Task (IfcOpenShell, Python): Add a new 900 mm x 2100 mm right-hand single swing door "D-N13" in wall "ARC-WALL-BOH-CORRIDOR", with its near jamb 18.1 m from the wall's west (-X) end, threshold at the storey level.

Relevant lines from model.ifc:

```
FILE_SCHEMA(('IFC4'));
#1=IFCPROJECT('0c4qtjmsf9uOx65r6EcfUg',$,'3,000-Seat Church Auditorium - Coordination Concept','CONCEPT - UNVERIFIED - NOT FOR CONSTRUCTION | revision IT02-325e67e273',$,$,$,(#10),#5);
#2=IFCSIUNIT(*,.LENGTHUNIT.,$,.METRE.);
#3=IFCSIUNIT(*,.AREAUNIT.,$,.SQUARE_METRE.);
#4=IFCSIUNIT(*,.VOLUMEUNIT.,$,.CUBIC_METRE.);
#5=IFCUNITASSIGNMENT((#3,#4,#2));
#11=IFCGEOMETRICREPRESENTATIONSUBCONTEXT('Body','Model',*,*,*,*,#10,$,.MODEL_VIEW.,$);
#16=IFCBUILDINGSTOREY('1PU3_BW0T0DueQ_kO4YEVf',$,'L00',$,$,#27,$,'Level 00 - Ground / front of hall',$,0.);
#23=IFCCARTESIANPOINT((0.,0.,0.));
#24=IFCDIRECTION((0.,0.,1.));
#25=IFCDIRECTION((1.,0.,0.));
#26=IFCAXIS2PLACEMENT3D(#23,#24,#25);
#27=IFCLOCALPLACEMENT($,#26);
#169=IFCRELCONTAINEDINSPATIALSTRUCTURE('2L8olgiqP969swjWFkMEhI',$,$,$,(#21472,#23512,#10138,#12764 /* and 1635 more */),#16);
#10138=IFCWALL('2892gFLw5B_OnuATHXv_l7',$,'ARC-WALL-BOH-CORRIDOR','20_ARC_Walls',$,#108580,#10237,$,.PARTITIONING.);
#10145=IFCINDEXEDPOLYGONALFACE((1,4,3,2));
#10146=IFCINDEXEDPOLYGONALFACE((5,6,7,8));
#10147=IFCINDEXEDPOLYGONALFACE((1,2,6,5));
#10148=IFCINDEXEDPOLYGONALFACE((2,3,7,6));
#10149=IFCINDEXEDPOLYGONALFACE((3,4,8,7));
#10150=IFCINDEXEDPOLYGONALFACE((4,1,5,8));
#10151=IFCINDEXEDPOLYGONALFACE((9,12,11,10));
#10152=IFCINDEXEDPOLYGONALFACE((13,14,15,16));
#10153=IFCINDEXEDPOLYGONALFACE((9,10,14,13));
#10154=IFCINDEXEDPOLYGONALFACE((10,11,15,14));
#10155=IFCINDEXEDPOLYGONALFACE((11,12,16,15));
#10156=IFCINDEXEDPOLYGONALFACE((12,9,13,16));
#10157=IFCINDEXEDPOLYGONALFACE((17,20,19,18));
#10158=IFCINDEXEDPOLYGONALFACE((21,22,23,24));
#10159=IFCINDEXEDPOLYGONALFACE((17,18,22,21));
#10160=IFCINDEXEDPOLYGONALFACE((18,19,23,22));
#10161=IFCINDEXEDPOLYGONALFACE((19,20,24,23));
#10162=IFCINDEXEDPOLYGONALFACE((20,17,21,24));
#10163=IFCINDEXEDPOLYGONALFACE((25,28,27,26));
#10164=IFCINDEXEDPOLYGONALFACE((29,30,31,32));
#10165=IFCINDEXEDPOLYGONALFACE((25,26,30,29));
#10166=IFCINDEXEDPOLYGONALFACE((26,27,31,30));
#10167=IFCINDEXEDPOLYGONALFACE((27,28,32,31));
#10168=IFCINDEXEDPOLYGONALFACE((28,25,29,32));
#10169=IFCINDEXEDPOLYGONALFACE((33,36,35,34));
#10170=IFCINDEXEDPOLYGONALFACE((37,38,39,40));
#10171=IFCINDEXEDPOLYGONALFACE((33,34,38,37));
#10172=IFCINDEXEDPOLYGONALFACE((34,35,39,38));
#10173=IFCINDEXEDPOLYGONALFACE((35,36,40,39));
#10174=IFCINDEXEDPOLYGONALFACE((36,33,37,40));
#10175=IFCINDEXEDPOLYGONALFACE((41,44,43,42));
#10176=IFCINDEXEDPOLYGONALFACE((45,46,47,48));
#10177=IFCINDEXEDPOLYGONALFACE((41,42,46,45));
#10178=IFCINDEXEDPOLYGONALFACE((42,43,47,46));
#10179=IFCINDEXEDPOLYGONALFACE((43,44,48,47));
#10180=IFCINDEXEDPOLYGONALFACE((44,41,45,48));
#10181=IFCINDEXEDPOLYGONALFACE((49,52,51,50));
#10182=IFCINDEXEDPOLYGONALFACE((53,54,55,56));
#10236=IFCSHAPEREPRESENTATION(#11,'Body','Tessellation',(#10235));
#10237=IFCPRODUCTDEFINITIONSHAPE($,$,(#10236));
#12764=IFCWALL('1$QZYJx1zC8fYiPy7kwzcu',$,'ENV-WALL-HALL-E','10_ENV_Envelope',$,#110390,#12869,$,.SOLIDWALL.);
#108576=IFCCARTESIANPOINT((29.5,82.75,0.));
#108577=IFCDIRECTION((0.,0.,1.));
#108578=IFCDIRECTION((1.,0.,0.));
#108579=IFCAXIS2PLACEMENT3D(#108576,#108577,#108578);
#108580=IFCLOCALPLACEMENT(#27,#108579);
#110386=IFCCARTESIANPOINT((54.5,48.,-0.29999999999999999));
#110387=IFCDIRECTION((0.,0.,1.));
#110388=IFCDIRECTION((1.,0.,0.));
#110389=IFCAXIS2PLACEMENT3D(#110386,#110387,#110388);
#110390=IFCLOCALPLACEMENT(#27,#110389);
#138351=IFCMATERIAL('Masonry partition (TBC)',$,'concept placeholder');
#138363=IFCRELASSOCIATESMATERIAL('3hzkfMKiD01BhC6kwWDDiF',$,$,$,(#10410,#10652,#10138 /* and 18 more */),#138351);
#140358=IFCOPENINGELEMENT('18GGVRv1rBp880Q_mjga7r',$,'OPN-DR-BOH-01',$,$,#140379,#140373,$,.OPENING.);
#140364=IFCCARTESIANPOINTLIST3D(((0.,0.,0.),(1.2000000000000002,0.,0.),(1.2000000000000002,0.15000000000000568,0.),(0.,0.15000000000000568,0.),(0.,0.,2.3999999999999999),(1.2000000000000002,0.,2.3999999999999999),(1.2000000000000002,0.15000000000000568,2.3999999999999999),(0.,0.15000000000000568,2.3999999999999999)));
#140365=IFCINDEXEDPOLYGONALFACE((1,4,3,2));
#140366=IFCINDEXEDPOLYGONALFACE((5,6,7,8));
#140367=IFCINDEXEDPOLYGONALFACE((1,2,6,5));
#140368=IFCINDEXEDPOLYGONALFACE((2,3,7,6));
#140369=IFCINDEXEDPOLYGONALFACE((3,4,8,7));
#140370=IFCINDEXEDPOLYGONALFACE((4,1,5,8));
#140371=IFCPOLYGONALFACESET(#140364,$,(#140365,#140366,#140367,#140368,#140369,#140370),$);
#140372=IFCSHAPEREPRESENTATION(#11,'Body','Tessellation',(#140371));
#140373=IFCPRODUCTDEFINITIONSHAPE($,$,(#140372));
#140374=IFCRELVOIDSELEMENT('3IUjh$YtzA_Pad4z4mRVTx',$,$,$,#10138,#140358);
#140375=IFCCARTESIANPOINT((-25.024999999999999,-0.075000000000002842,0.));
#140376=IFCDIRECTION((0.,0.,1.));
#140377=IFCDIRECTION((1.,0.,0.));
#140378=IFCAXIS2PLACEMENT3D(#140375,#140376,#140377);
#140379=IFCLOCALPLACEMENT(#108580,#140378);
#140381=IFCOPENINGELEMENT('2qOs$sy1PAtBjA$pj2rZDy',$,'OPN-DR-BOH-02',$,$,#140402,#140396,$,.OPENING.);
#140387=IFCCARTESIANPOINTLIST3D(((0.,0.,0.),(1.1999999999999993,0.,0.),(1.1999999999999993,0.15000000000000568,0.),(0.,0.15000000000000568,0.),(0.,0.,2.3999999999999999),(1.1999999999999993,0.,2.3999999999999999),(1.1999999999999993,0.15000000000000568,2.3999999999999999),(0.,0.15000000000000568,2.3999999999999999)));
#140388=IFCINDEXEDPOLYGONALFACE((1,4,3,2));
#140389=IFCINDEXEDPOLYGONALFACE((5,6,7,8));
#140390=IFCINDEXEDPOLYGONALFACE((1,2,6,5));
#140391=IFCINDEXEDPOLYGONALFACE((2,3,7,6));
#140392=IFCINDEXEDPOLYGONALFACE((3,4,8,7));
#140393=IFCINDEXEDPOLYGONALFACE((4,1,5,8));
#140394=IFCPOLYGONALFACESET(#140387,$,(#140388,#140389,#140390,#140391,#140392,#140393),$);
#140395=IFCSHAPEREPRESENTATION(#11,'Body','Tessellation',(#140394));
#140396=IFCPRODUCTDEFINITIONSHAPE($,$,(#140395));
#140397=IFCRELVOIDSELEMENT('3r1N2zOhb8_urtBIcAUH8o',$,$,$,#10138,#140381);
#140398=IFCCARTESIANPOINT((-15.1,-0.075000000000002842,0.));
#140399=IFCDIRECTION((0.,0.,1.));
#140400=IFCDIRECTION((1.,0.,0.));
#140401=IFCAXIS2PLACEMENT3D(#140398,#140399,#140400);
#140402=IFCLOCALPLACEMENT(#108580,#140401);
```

```python
import numpy as np
import ifcopenshell
import ifcopenshell.api.feature
import ifcopenshell.api.geometry
import ifcopenshell.api.root
import ifcopenshell.api.spatial
import ifcopenshell.geom
import ifcopenshell.util.element
import ifcopenshell.util.placement
import ifcopenshell.util.representation
import ifcopenshell.util.shape
import ifcopenshell.util.unit

model = ifcopenshell.open("model.ifc")
unit_scale = ifcopenshell.util.unit.calculate_unit_scale(model)
settings = ifcopenshell.geom.settings()


def volume(element):
    """Net volume in cubic metres, openings subtracted."""
    shape = ifcopenshell.geom.create_shape(settings, element)
    return ifcopenshell.util.shape.get_volume(shape.geometry)


wall = model.by_id(10138)
storey = ifcopenshell.util.element.get_container(wall, ifc_class="IfcBuildingStorey")
context = ifcopenshell.util.representation.get_context(model, "Model", "Body", "MODEL_VIEW")
before = volume(wall)

width, height, from_end, sill = 0.9, 2.1, 18.1, 0.0  # metres

# The wall runs along its own X axis, and the end named is its -X end.
wall_shape = ifcopenshell.geom.create_shape(settings, wall)
x, y, z = ifcopenshell.util.shape.get_vertices(wall_shape.geometry).T
start = x.min() + from_end
face, thickness = float(y.min()), float(y.max() - y.min())
wall_matrix = ifcopenshell.util.placement.get_local_placement(wall.ObjectPlacement)
level = ifcopenshell.util.placement.get_local_placement(storey.ObjectPlacement)[2, 3]


def in_wall(x, y):
    """Placement at x, y metres in the wall's axes, at sill height."""
    matrix = wall_matrix.copy()
    matrix[:, 3] = wall_matrix @ np.array([x / unit_scale, y / unit_scale, 0.0, 1.0])
    matrix[2, 3] = level + sill / unit_scale
    return matrix


# Opening: a box that overshoots both wall faces by 50 mm.
opening = ifcopenshell.api.root.create_entity(model, ifc_class="IfcOpeningElement", predefined_type="OPENING")
box = ifcopenshell.api.geometry.add_wall_representation(
    model, context=context, length=width, height=height, thickness=thickness + 0.1
)
ifcopenshell.api.geometry.assign_representation(model, product=opening, representation=box)
ifcopenshell.api.geometry.edit_object_placement(model, product=opening, matrix=in_wall(start, face - 0.05), is_si=False)
ifcopenshell.api.feature.add_feature(model, feature=opening, element=wall)

door = ifcopenshell.api.root.create_entity(model, ifc_class="IfcDoor", name="D-N13", predefined_type="DOOR")
door.OverallWidth, door.OverallHeight = width / unit_scale, height / unit_scale
door.OperationType = "SINGLE_SWING_RIGHT"
body = ifcopenshell.api.geometry.add_door_representation(
    model,
    context=context,
    overall_width=door.OverallWidth,
    overall_height=door.OverallHeight,
    operation_type="SINGLE_SWING_RIGHT",
    lining_properties={"LiningDepth": thickness / unit_scale, "ThresholdDepth": thickness / unit_scale},
)
ifcopenshell.api.geometry.assign_representation(model, product=door, representation=body)
ifcopenshell.api.spatial.assign_container(model, products=[door], relating_structure=storey)
ifcopenshell.api.feature.add_filling(model, opening=opening, element=door)

# The lining spans the wall, so the door starts at the wall face.
ifcopenshell.api.geometry.edit_object_placement(model, product=door, matrix=in_wall(start, face), is_si=False)

after = volume(wall)

print(f"wall volume {before:.3f} -> {after:.3f} m3")

model.write("model_rev.ifc")
```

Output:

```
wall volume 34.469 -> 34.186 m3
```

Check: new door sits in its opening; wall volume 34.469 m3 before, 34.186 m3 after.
